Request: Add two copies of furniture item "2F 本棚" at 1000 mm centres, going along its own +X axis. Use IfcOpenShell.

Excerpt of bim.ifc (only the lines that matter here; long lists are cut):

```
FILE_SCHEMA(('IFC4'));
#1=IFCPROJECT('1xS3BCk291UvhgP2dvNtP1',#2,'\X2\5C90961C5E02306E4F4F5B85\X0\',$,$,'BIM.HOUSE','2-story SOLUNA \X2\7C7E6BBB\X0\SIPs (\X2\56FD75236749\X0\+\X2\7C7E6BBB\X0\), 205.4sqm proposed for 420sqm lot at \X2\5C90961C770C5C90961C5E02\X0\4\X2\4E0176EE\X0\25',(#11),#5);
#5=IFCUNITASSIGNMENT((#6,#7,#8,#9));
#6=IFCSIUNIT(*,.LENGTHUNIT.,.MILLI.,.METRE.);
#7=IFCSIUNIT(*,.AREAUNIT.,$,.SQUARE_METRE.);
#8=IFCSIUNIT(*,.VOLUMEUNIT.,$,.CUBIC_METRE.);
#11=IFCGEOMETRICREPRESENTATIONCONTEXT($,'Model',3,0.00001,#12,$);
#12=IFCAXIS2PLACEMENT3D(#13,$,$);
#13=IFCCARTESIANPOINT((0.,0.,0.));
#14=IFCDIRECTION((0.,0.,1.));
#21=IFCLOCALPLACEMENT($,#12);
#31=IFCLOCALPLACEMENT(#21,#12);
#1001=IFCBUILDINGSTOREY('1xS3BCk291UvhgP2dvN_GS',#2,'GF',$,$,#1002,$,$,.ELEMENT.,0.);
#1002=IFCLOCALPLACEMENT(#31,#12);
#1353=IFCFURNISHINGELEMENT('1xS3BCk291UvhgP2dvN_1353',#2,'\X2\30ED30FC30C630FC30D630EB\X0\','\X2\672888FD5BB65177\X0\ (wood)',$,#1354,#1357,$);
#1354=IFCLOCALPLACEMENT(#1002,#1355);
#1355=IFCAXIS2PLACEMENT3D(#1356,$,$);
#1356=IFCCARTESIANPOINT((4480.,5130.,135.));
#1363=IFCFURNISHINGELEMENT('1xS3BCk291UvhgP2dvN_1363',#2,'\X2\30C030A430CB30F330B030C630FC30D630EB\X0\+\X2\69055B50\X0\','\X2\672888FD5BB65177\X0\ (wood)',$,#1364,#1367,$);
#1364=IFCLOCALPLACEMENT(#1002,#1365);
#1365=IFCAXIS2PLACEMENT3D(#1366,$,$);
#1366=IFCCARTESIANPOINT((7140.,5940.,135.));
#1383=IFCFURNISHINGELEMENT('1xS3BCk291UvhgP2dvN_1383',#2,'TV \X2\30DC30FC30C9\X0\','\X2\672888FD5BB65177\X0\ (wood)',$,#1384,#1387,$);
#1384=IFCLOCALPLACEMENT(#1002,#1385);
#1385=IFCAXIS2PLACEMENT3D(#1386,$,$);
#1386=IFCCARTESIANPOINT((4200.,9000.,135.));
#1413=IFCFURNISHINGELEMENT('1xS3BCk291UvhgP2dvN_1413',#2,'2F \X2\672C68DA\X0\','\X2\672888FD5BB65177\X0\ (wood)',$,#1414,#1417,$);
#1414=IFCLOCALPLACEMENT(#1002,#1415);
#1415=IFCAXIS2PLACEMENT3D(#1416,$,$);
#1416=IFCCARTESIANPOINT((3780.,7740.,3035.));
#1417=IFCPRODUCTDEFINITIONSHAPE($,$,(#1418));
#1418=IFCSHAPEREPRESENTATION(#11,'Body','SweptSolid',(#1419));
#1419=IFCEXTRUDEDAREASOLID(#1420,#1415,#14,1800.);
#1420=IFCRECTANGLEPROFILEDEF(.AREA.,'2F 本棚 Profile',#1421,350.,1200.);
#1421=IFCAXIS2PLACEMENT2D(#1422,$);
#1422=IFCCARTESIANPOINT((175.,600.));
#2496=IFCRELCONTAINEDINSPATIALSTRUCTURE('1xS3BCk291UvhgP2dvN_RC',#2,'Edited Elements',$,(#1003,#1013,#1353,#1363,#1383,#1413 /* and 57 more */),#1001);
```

```python
import ifcopenshell
import ifcopenshell.api.geometry
import ifcopenshell.api.root
import ifcopenshell.util.element
import ifcopenshell.util.placement
import ifcopenshell.util.unit

model = ifcopenshell.open("bim.ifc")
unit_scale = ifcopenshell.util.unit.calculate_unit_scale(model)


def reuse_history(source, copy):
    """copy_class also copies each property set's owner history, people and application; keep the originals."""
    for rel in copy.IsDefinedBy:
        if rel.is_a("IfcRelDefinesByProperties") and (history := rel.RelatingPropertyDefinition.OwnerHistory):
            rel.RelatingPropertyDefinition.OwnerHistory = source.OwnerHistory
            ifcopenshell.util.element.remove_deep2(model, history)


source = model.by_id(1413)
base = ifcopenshell.util.placement.get_local_placement(source.ObjectPlacement)
step = base[:3, 0] * 1 / unit_scale

for i in range(1, 3):
    copy = ifcopenshell.api.root.copy_class(model, product=source)
    copy.Representation = ifcopenshell.util.element.copy_deep(
        model, source.Representation, exclude=["IfcGeometricRepresentationContext", "IfcRepresentationMap"]
    )
    reuse_history(source, copy)
    matrix = base.copy()
    matrix[:3, 3] += i * step
    print("added at", matrix[:3, 3].round(3) + 0.0)
    ifcopenshell.api.geometry.edit_object_placement(model, product=copy, matrix=matrix, is_si=False)

model.write("bim_updated.ifc")
```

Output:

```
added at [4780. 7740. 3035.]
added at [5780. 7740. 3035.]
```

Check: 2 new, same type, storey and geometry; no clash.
